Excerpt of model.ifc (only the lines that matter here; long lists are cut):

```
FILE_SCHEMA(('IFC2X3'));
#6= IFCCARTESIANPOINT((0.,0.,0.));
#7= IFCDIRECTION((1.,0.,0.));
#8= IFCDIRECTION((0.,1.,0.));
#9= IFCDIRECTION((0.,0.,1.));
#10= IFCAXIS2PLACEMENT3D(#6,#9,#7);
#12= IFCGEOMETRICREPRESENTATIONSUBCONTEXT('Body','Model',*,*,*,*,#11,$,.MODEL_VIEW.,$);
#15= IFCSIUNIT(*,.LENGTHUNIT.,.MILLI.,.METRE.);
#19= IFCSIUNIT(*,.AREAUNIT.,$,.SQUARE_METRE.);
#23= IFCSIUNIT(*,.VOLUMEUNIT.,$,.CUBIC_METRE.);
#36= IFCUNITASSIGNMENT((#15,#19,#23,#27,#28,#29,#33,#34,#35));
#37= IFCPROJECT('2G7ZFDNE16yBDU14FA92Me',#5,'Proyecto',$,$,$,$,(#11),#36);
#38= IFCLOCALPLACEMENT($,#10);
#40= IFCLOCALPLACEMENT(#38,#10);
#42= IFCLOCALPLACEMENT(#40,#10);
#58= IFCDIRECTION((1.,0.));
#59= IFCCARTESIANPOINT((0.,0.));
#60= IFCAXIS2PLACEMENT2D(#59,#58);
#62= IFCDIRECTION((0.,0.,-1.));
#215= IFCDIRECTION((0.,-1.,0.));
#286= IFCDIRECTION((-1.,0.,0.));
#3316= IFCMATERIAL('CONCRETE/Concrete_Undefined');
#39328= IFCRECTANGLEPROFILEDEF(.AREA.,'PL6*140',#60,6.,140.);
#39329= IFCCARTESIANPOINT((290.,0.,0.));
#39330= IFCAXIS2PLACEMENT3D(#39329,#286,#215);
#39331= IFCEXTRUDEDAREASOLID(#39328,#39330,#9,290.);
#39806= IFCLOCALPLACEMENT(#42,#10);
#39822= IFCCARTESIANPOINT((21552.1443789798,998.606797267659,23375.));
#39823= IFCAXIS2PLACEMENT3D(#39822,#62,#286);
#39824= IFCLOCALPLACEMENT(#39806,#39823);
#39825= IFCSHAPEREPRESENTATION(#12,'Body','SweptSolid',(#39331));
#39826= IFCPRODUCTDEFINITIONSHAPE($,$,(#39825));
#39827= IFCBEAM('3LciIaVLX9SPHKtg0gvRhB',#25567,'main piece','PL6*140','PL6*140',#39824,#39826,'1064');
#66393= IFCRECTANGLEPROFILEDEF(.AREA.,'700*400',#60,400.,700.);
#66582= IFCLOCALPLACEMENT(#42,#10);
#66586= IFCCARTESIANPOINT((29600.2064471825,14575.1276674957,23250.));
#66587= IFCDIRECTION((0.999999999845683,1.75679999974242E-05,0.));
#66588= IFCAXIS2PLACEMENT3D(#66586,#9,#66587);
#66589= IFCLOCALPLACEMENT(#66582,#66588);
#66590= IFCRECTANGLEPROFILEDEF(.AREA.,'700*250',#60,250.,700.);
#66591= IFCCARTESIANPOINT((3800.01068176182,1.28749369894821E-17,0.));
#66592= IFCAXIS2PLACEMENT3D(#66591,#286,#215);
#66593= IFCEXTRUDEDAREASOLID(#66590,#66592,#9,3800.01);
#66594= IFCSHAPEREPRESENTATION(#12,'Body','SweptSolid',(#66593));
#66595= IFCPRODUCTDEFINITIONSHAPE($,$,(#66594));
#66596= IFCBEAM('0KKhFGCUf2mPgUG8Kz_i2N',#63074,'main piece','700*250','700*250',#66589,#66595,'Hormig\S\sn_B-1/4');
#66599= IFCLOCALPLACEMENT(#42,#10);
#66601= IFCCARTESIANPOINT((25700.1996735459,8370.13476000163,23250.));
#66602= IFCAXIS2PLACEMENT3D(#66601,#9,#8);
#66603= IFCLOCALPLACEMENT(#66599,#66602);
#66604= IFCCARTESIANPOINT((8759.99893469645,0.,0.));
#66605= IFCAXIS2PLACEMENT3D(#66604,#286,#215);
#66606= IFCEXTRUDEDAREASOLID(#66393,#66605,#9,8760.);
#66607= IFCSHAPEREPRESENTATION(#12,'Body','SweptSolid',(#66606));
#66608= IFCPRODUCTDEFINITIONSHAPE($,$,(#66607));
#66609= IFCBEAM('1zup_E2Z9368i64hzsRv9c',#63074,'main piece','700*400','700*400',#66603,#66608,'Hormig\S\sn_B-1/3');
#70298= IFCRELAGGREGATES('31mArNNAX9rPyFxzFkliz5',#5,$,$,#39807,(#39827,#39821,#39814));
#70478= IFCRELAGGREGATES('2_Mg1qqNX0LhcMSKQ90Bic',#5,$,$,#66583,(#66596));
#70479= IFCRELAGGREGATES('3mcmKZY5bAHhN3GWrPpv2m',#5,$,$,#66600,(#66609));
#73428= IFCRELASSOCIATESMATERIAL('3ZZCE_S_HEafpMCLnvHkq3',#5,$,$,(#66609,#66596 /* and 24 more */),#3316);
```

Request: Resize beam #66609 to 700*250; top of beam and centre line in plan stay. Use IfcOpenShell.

```python
import ifcopenshell
import ifcopenshell.util.element
import ifcopenshell.util.representation

model = ifcopenshell.open("model.ifc")

member = model.by_id(66609)
source = next(p for p in model.by_type("IfcRectangleProfileDef") if p.ProfileName == "700*250")

body = ifcopenshell.util.representation.get_representation(member, "Model", "Body")
solid = body.Items[0]
old_profile = solid.SweptArea

# Copy the section's sizes but keep this member's own profile position.
profile = ifcopenshell.util.element.copy(model, source)
# Profiles are centred, so shift by half the change in depth to hold the top.
shift = (old_profile.YDim - profile.YDim) / 2
x, y = old_profile.Position.Location.Coordinates
up = (0.0, 1.0)  # upwards, in the solid's own plane
location = model.createIfcCartesianPoint((x + up[0] * shift, y + up[1] * shift))
profile.Position = model.createIfcAxis2Placement2D(location, old_profile.Position.RefDirection)
solid.SweptArea = profile
if not model.get_total_inverses(old_profile):
    ifcopenshell.util.element.remove_deep2(model, old_profile)
member.Description = member.Description.replace("700*400", "700*250")
member.ObjectType = member.ObjectType.replace("700*400", "700*250")

print(solid.SweptArea)

model.write("model_v2.ifc")
```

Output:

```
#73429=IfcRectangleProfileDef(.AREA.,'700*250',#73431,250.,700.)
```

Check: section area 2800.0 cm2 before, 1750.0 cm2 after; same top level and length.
